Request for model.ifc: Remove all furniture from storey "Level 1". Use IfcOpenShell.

First a look at what the model holds.

```python
import ifcopenshell
import ifcopenshell.util.element

model = ifcopenshell.open("model.ifc")
print(model.schema)
storey = next(s for s in model.by_type("IfcBuildingStorey") if s.Name == "Level 1")
furniture = [e for e in ifcopenshell.util.element.get_decomposition(storey) if e.is_a("IfcFurnishingElement")]
seen = {}
for e in furniture:
    element_type = ifcopenshell.util.element.get_type(e)
    name = element_type.Name if element_type not in (None, e) else None
    seen[name] = seen.get(name, 0) + 1
for name, count in sorted(seen.items(), key=str):
    print(count, "x", name)
```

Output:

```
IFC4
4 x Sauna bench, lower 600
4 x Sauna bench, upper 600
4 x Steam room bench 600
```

```python
import ifcopenshell
import ifcopenshell.api.root
import ifcopenshell.util.element

model = ifcopenshell.open("model.ifc")

storey = next(s for s in model.by_type("IfcBuildingStorey") if s.Name == "Level 1")
furniture = [e for e in ifcopenshell.util.element.get_decomposition(storey) if e.is_a("IfcFurnishingElement")]

for e in furniture:
    ifcopenshell.api.root.remove_product(model, product=e)
print(len(furniture), "removed")

model.write("model_updated.ifc")
```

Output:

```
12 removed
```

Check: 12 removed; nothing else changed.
